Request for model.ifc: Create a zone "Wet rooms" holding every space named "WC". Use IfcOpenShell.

First a look at what the model holds.

```python
import ifcopenshell

model = ifcopenshell.open("model.ifc")
print(model.schema)
seen = {}
for space in model.by_type("IfcSpace"):
    seen[space.LongName] = seen.get(space.LongName, 0) + 1
for name, count in sorted(seen.items(), key=str):
    print(count, "x", name)
print("zones:", [z.Name for z in model.by_type("IfcZone")][:20])
```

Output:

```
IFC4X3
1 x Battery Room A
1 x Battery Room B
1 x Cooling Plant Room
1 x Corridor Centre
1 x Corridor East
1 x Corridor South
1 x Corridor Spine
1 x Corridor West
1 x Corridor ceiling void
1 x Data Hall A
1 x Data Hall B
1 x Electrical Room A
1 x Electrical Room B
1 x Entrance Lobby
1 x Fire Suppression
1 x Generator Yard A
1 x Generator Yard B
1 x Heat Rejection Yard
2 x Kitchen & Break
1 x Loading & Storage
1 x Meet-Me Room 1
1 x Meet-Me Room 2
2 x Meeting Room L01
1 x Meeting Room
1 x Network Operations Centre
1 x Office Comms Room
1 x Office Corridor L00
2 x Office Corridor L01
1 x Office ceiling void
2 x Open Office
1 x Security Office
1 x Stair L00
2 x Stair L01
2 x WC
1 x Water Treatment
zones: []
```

```python
import ifcopenshell
import ifcopenshell.api.group
import ifcopenshell.api.root

model = ifcopenshell.open("model.ifc")

names = {"WC"}
spaces = [s for s in model.by_type("IfcSpace") if s.LongName in names]

zone = ifcopenshell.api.root.create_entity(model, ifc_class="IfcZone", name="Wet rooms")
ifcopenshell.api.group.assign_group(model, products=spaces, group=zone)
print(len(spaces), "spaces in", zone.Name)

model.write("model_v2.ifc")
```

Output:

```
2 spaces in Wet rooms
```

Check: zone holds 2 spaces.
